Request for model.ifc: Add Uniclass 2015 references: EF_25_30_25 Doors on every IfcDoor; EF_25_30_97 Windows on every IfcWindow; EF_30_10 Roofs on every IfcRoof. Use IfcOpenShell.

First a look at what the model holds.

```python
import ifcopenshell

model = ifcopenshell.open("model.ifc")
print(model.schema)
print("classifications:", [c.Name for c in model.by_type("IfcClassification")])
for ifc_class in ("IfcDoor", "IfcRoof", "IfcStair", "IfcWall", "IfcWindow"):
    print(ifc_class, len(model.by_type(ifc_class)))
```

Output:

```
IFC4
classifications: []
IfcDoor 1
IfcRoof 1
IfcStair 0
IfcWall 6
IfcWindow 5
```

```python
import ifcopenshell
import ifcopenshell.api.classification

model = ifcopenshell.open("model.ifc")

system = ifcopenshell.api.classification.add_classification(model, classification="Uniclass 2015")

codes = {
    "IfcDoor": ("EF_25_30_25", "Doors"),
    "IfcWindow": ("EF_25_30_97", "Windows"),
    "IfcRoof": ("EF_30_10", "Roofs"),
}
for ifc_class, (code, name) in codes.items():
    products = model.by_type(ifc_class)
    ifcopenshell.api.classification.add_reference(
        model, products=products, classification=system, identification=code, name=name
    )
    print(code, len(products))

model.write("model_updated.ifc")
```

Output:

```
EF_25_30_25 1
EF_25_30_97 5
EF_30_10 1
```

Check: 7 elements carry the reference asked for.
